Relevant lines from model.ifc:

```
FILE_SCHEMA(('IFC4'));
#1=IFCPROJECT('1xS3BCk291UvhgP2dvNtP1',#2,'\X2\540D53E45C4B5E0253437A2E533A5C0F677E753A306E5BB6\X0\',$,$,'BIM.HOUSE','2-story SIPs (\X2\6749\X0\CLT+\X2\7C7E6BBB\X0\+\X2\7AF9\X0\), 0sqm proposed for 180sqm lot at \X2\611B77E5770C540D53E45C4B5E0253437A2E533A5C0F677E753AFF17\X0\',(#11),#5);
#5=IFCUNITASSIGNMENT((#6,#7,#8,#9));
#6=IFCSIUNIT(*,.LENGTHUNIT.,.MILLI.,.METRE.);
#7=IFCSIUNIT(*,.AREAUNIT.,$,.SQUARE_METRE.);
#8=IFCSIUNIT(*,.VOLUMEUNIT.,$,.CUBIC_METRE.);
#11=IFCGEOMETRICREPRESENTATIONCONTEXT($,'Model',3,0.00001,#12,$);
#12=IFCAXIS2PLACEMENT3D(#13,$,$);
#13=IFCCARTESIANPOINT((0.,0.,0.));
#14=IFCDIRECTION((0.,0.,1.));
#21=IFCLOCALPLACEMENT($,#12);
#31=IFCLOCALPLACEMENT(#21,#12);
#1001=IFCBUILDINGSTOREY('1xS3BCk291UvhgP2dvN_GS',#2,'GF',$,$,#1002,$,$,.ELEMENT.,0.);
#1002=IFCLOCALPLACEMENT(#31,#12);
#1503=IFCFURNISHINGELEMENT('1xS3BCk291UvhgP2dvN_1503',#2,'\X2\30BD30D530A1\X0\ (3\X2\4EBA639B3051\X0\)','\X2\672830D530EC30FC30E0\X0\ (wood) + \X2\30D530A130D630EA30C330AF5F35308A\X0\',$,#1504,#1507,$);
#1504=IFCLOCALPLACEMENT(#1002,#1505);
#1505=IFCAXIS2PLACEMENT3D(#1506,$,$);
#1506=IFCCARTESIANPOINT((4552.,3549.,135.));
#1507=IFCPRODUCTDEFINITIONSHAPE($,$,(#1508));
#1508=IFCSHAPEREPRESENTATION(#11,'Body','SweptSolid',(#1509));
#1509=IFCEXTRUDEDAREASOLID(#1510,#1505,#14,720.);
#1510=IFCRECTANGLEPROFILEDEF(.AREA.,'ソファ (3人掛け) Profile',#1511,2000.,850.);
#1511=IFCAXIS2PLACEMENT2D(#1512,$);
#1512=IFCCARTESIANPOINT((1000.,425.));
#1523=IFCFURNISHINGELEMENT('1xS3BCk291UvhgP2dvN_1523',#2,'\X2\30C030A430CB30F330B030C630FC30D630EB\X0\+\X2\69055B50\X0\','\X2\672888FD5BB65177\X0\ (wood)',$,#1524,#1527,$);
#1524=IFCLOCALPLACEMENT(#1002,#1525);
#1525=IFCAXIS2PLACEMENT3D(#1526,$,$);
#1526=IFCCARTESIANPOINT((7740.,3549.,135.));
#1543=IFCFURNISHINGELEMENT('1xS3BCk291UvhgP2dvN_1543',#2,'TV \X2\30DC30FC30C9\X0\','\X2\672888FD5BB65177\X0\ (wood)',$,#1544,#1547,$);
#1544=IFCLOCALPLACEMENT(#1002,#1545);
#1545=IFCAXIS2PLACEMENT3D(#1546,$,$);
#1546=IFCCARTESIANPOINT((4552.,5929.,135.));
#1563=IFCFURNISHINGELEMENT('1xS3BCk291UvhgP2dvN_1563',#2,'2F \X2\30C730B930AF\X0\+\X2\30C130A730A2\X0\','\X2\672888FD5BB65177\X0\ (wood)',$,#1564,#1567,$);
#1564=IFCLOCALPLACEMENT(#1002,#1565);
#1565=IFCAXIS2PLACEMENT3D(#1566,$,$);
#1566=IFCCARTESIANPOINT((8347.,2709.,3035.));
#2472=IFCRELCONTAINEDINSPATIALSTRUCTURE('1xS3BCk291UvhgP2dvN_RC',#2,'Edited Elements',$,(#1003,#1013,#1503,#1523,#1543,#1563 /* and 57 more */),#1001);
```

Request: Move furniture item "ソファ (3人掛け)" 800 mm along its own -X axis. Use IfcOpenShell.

```python
import ifcopenshell
import ifcopenshell.api.geometry
import ifcopenshell.util.placement

model = ifcopenshell.open("model.ifc")

item = model.by_guid("1xS3BCk291UvhgP2dvN_1503")
matrix = ifcopenshell.util.placement.get_local_placement(item.ObjectPlacement)
matrix[:3, 3] -= matrix[:3, 0] * 800.0
ifcopenshell.api.geometry.edit_object_placement(model, product=item, matrix=matrix, is_si=False)

print(ifcopenshell.util.placement.get_local_placement(item.ObjectPlacement).round(3) + 0.0)

model.write("model_edited.ifc")
```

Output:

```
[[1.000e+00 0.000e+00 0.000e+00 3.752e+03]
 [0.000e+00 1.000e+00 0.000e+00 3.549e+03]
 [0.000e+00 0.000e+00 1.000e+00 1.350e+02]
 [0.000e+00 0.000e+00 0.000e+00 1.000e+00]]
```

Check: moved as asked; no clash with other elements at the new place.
